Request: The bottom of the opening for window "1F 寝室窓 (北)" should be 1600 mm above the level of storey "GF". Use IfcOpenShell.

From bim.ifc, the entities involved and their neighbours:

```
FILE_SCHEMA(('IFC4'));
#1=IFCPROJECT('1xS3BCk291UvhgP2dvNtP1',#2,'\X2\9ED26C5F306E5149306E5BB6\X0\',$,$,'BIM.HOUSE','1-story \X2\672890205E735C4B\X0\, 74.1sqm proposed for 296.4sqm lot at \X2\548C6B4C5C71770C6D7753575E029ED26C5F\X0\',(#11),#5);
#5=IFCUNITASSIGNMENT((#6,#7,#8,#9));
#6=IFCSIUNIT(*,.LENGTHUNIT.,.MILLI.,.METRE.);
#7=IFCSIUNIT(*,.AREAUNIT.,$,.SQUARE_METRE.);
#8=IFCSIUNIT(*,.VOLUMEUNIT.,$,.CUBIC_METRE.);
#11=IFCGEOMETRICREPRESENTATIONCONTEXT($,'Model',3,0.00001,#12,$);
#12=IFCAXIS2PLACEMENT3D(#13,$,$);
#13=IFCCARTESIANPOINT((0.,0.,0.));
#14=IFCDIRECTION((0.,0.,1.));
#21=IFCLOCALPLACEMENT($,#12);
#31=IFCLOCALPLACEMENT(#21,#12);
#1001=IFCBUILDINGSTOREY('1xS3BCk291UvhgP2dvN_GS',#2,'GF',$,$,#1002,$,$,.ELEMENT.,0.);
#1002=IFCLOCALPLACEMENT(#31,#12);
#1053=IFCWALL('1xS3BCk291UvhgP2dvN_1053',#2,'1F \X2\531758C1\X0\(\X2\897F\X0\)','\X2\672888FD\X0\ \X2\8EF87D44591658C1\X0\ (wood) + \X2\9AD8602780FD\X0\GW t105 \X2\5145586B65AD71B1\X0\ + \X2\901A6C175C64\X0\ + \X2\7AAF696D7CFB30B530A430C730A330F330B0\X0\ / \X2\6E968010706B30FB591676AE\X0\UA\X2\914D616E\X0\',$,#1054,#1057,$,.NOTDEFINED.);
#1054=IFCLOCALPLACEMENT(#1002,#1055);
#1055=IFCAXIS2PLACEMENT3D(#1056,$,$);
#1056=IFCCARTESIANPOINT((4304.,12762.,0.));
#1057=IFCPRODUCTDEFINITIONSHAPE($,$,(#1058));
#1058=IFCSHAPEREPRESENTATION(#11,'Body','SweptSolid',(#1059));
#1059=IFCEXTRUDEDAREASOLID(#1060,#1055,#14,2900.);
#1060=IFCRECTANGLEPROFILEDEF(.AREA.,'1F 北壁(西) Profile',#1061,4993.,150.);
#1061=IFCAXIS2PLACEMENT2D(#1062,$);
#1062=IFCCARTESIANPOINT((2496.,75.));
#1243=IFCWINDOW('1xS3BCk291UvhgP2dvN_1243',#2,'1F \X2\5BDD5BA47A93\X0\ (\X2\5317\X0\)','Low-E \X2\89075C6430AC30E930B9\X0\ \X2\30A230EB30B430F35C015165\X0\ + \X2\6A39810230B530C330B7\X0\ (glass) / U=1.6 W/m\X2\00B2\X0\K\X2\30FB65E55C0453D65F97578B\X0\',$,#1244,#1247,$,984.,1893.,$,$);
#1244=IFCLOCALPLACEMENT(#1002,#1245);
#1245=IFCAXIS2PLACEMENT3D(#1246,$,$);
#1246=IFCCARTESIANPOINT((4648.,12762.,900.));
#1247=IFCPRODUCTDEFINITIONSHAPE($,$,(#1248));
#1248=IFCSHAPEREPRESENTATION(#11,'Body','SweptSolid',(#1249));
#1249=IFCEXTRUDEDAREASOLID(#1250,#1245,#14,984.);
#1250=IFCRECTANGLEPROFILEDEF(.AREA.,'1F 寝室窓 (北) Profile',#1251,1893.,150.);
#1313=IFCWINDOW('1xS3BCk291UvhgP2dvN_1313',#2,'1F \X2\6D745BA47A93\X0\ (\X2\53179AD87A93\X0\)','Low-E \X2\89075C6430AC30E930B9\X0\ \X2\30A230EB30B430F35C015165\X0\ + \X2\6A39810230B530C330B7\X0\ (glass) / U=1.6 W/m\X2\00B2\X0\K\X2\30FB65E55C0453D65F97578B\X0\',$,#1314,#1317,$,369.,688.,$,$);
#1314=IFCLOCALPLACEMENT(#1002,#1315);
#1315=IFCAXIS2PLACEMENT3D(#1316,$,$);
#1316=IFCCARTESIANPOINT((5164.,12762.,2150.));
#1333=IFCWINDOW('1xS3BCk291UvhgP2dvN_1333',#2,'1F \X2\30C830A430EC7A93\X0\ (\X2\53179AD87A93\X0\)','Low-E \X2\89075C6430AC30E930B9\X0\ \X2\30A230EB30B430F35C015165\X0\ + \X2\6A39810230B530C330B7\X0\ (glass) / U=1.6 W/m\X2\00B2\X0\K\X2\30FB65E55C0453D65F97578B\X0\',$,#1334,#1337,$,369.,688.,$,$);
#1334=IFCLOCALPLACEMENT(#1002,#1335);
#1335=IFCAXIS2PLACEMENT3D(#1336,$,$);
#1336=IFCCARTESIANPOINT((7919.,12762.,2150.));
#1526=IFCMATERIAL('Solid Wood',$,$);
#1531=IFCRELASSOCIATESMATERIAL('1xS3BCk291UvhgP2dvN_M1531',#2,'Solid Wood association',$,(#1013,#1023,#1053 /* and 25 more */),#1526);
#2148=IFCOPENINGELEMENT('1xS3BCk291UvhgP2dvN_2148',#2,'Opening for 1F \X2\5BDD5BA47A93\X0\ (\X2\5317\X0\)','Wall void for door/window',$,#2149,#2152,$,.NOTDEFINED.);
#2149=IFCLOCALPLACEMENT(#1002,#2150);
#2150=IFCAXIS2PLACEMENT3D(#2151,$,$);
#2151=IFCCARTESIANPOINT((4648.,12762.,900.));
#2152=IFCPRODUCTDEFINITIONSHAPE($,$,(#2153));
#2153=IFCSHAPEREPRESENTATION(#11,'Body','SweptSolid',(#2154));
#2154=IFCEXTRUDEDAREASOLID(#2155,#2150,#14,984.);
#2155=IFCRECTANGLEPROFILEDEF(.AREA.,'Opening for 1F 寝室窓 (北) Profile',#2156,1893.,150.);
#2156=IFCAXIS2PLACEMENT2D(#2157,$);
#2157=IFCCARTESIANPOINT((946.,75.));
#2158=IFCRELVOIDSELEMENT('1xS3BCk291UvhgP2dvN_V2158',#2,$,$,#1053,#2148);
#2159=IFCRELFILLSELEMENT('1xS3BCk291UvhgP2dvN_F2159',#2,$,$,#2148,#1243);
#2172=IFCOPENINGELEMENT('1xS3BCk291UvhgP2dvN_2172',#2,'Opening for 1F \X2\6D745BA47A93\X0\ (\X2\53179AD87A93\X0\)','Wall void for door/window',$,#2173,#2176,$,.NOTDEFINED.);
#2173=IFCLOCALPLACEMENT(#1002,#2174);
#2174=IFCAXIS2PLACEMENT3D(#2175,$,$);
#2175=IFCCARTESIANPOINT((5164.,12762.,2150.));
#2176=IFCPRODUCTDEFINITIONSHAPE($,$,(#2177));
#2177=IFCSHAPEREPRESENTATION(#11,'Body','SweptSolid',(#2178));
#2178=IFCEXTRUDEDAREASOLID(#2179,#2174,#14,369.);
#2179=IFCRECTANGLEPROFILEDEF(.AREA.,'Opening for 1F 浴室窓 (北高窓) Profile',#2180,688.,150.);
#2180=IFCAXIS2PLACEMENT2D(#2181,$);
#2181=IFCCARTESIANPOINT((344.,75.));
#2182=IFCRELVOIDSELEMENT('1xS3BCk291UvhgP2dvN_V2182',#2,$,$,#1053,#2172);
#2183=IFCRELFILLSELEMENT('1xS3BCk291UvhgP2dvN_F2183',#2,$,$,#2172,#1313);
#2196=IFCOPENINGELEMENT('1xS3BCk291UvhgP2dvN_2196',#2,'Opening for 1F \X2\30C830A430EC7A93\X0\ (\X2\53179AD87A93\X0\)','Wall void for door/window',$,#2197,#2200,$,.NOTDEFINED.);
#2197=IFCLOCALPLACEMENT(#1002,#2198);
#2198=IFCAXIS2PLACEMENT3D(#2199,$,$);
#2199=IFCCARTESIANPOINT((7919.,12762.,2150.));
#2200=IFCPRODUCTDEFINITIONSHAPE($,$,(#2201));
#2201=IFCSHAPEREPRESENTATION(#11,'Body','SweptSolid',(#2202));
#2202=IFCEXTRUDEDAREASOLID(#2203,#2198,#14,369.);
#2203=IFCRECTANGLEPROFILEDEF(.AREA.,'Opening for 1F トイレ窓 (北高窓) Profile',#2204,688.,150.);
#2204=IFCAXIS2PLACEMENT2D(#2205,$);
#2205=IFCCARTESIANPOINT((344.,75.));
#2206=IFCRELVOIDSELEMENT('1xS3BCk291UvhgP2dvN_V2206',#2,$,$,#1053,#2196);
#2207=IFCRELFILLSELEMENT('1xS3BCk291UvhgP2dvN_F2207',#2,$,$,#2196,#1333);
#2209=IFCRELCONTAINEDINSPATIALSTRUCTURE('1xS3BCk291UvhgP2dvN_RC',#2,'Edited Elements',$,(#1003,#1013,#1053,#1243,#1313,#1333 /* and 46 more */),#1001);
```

```python
import numpy as np
import ifcopenshell
import ifcopenshell.api.geometry
import ifcopenshell.geom
import ifcopenshell.util.element
import ifcopenshell.util.placement
import ifcopenshell.util.shape
import ifcopenshell.util.unit

model = ifcopenshell.open("bim.ifc")
unit_scale = ifcopenshell.util.unit.calculate_unit_scale(model)

window = model.by_guid("1xS3BCk291UvhgP2dvN_1243")
opening = window.FillsVoids[0].RelatingOpeningElement
storey = ifcopenshell.util.element.get_container(window, ifc_class="IfcBuildingStorey")
level = ifcopenshell.util.placement.get_local_placement(storey.ObjectPlacement)[2, 3]

# The opening's origin need not be at the sill, so measure its lowest point.
shape = ifcopenshell.geom.create_shape(ifcopenshell.geom.settings(), opening)
bottom = ifcopenshell.util.shape.get_shape_bottom_elevation(shape, shape.geometry) / unit_scale
dz = level + 1600.0 - bottom

shift = np.array([0.0, 0.0, dz])
# The window is not placed relative to its opening, so move both.
for product in (opening, window):
    matrix = ifcopenshell.util.placement.get_local_placement(product.ObjectPlacement)
    matrix[:3, 3] += shift
    ifcopenshell.api.geometry.edit_object_placement(model, product=product, matrix=matrix, is_si=False)

print(f"moved by {dz * unit_scale:+.3f} m")

model.write("bim_rev.ifc")
```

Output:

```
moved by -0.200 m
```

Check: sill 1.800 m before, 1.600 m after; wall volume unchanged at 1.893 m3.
